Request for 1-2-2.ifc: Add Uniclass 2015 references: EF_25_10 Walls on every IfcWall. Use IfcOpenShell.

First a look at what the model holds.

```python
import ifcopenshell

model = ifcopenshell.open("1-2-2.ifc")
print(model.schema)
print("classifications:", [c.Name for c in model.by_type("IfcClassification")])
for ifc_class in ("IfcDoor", "IfcRoof", "IfcStair", "IfcWall", "IfcWindow"):
    print(ifc_class, len(model.by_type(ifc_class)))
```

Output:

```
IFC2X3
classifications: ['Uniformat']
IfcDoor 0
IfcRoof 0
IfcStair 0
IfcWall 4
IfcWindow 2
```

```python
import ifcopenshell
import ifcopenshell.api.classification

model = ifcopenshell.open("1-2-2.ifc")

# IFC2X3 requires Source and Edition and has no link from the project to the system.
system = model.create_entity("IfcClassification", Source="NBS", Edition="2015", Name="Uniclass 2015")

codes = {
    "IfcWall": ("EF_25_10", "Walls"),
}
for ifc_class, (code, name) in codes.items():
    products = model.by_type(ifc_class)
    ifcopenshell.api.classification.add_reference(
        model, products=products, classification=system, identification=code, name=name
    )
    print(code, len(products))

model.write("1-2-2-out.ifc")
```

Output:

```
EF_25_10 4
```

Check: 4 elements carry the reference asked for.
